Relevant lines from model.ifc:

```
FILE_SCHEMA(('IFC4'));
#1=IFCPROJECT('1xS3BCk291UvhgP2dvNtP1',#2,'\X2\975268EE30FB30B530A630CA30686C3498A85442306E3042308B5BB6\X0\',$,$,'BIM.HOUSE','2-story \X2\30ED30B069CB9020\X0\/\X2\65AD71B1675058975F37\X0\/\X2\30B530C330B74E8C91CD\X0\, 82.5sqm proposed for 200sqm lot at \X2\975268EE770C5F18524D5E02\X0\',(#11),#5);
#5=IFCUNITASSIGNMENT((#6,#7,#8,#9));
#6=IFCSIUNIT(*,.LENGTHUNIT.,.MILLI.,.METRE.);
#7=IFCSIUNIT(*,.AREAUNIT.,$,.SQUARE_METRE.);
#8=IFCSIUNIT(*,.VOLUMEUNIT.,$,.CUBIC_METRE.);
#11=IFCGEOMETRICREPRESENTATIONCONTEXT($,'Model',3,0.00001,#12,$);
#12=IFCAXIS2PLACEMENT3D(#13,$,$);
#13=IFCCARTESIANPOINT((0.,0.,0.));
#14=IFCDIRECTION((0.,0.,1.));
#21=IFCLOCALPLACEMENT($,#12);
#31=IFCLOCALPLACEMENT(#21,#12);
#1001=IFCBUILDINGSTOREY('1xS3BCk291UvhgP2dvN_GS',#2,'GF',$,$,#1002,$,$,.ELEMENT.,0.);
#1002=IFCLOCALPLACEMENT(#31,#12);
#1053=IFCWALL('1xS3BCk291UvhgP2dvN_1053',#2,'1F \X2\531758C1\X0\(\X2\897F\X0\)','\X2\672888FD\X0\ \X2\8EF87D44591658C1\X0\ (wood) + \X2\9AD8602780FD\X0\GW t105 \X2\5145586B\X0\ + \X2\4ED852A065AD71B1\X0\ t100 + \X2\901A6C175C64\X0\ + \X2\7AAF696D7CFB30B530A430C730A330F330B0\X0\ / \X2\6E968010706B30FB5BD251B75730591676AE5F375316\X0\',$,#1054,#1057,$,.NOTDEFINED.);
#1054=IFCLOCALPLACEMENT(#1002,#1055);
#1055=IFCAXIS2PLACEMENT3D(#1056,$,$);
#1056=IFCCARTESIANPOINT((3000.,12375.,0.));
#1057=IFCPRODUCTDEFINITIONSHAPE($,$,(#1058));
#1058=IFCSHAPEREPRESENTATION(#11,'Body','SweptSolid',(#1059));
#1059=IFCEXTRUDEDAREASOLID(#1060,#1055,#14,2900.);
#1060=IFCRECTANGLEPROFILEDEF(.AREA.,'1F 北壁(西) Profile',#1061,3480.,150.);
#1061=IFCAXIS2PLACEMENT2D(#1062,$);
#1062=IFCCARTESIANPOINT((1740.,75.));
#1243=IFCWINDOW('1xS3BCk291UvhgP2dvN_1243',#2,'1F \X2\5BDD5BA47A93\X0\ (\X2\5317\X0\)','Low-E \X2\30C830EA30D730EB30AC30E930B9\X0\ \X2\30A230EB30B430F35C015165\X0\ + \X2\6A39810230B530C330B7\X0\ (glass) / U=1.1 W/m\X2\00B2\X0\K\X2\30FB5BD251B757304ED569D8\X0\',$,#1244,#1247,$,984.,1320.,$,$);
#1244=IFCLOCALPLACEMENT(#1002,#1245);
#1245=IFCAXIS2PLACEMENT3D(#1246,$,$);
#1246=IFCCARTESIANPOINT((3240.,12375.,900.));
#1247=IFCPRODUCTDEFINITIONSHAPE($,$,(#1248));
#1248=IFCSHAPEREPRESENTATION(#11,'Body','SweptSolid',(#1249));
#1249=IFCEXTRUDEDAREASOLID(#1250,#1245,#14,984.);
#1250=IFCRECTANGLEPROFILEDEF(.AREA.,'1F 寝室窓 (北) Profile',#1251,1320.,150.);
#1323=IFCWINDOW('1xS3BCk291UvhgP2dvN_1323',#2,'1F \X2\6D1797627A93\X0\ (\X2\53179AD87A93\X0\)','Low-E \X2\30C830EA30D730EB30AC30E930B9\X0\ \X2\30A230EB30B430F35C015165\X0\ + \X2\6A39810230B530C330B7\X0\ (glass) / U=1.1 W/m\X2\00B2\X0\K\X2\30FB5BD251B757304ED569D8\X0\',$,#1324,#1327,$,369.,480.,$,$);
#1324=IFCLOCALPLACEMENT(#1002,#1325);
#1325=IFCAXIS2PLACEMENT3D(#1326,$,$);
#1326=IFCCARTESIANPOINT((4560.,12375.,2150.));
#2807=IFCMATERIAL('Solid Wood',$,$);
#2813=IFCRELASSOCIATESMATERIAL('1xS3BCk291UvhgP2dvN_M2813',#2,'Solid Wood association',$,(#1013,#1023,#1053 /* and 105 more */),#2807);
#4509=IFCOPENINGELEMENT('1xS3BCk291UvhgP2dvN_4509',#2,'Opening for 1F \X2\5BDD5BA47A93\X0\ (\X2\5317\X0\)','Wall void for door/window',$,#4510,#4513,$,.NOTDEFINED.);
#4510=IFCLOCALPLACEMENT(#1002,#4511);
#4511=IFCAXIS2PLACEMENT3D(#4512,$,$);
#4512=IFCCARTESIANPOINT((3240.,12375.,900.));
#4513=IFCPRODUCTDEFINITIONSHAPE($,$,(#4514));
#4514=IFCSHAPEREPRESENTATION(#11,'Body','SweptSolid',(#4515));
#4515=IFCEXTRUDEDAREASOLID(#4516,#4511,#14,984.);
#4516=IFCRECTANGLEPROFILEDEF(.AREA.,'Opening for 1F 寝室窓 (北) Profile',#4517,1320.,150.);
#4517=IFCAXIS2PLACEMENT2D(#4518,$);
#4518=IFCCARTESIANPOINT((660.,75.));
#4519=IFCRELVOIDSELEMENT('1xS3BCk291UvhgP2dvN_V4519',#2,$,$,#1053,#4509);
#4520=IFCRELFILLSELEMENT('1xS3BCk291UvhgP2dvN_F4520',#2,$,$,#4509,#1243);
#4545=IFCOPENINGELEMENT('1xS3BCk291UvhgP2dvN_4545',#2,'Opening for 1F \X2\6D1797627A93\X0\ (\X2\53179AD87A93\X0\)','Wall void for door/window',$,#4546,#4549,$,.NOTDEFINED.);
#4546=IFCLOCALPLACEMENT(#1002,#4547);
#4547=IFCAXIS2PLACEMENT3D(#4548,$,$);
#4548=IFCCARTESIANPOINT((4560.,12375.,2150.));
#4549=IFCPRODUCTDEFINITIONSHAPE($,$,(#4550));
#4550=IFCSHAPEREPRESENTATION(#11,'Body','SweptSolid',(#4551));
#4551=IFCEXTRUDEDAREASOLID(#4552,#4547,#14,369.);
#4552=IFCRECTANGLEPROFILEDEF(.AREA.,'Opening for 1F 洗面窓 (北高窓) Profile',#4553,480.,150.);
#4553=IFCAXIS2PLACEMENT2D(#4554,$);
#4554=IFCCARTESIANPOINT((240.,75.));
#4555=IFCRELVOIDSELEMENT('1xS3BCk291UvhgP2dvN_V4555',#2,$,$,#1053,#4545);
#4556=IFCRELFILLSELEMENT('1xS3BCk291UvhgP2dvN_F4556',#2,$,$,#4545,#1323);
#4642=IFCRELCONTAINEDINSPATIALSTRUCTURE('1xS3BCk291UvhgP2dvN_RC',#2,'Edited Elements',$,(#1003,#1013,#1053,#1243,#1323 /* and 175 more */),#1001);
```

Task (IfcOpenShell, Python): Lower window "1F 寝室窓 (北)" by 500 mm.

```python
import numpy as np
import ifcopenshell
import ifcopenshell.api.geometry
import ifcopenshell.util.placement
import ifcopenshell.util.unit

model = ifcopenshell.open("model.ifc")
unit_scale = ifcopenshell.util.unit.calculate_unit_scale(model)

window = model.by_id(1243)
opening = window.FillsVoids[0].RelatingOpeningElement
dz = -0.5 / unit_scale

shift = np.array([0.0, 0.0, dz])
# The window is not placed relative to its opening, so move both.
for product in (opening, window):
    matrix = ifcopenshell.util.placement.get_local_placement(product.ObjectPlacement)
    matrix[:3, 3] += shift
    ifcopenshell.api.geometry.edit_object_placement(model, product=product, matrix=matrix, is_si=False)

print(f"moved by {dz * unit_scale:+.3f} m")

model.write("model_edited.ifc")
```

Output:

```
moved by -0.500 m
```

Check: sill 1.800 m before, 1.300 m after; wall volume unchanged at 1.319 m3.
